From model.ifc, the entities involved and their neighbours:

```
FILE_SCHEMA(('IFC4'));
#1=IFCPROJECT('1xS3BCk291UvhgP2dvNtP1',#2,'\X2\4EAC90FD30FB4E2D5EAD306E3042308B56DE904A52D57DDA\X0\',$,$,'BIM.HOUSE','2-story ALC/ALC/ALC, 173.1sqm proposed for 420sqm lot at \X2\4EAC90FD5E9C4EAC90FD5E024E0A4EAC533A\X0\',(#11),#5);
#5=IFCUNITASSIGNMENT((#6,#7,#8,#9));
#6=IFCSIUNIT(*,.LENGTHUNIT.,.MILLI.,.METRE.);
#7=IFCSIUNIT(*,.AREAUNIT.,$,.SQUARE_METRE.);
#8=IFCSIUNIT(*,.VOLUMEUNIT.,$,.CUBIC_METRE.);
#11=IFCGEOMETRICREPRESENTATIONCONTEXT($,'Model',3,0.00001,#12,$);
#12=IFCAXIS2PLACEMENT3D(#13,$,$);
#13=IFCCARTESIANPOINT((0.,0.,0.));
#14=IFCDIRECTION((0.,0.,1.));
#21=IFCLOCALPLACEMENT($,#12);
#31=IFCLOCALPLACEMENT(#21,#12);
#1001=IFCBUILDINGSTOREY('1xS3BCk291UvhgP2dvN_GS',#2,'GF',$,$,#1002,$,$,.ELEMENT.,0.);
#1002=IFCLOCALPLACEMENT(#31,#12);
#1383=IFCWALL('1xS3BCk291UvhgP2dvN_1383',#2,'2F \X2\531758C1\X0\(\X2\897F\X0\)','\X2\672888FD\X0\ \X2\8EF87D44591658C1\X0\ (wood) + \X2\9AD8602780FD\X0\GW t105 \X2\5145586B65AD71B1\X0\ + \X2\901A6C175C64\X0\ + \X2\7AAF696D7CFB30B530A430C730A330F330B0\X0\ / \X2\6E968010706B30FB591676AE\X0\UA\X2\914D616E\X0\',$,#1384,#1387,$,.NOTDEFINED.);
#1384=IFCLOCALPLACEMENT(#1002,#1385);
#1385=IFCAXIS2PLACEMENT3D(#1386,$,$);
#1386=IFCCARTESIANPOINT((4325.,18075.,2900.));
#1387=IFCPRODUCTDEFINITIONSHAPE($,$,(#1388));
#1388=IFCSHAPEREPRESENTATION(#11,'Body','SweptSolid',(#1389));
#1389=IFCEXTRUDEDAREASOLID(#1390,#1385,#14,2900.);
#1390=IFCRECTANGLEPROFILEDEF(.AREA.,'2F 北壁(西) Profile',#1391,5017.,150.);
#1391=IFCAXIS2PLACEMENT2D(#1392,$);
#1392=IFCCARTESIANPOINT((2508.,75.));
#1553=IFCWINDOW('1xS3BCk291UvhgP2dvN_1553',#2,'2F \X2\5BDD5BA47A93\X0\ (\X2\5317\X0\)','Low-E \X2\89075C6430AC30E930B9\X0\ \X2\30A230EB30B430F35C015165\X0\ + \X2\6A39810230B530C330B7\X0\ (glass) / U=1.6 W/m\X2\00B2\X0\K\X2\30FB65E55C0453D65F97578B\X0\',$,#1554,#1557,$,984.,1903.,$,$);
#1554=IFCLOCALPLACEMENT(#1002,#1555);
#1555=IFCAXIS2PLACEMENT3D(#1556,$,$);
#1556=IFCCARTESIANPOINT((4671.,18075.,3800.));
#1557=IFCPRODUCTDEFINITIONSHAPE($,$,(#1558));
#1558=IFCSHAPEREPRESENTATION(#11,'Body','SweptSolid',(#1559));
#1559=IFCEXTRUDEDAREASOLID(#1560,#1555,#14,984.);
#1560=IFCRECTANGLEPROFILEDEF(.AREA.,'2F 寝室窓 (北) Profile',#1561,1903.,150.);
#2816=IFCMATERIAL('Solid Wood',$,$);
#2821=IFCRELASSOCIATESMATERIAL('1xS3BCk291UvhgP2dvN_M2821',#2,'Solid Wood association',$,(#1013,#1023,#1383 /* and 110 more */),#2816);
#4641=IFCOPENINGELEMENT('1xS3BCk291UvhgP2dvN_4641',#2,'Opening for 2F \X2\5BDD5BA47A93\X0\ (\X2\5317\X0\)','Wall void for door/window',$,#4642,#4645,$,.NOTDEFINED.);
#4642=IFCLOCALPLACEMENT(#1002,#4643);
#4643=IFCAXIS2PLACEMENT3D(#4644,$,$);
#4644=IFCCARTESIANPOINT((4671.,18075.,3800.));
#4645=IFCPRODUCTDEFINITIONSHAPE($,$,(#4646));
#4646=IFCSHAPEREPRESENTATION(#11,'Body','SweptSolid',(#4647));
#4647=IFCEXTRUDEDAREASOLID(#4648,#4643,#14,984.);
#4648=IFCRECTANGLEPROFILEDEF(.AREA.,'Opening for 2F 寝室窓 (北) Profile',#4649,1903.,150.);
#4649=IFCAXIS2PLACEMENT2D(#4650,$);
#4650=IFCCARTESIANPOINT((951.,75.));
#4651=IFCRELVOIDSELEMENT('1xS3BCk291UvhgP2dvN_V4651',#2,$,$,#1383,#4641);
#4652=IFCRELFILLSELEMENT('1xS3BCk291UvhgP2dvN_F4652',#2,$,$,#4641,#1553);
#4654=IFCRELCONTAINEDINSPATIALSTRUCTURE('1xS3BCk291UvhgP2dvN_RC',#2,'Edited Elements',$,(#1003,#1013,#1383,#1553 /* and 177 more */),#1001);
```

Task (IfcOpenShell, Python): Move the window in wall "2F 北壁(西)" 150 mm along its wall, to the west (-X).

```python
import ifcopenshell
import ifcopenshell.api.geometry
import ifcopenshell.util.placement

model = ifcopenshell.open("model.ifc")

window = model.by_guid("1xS3BCk291UvhgP2dvN_1553")
opening = window.FillsVoids[0].RelatingOpeningElement
wall = opening.VoidsElements[0].RelatingBuildingElement

wall_matrix = ifcopenshell.util.placement.get_local_placement(wall.ObjectPlacement)
shift = wall_matrix[:3, 0] * -150.0
before = ifcopenshell.util.placement.get_local_placement(window.ObjectPlacement)[:3, 3].copy()

# The window is not placed relative to its opening, so move both.
for product in (opening, window):
    matrix = ifcopenshell.util.placement.get_local_placement(product.ObjectPlacement)
    matrix[:3, 3] += shift
    ifcopenshell.api.geometry.edit_object_placement(model, product=product, matrix=matrix, is_si=False)

after = ifcopenshell.util.placement.get_local_placement(window.ObjectPlacement)[:3, 3]
print("window moved by", (after - before).round(3) + 0.0)

model.write("model_v2.ifc")
```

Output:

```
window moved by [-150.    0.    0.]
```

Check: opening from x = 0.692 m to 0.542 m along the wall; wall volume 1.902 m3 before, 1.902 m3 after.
